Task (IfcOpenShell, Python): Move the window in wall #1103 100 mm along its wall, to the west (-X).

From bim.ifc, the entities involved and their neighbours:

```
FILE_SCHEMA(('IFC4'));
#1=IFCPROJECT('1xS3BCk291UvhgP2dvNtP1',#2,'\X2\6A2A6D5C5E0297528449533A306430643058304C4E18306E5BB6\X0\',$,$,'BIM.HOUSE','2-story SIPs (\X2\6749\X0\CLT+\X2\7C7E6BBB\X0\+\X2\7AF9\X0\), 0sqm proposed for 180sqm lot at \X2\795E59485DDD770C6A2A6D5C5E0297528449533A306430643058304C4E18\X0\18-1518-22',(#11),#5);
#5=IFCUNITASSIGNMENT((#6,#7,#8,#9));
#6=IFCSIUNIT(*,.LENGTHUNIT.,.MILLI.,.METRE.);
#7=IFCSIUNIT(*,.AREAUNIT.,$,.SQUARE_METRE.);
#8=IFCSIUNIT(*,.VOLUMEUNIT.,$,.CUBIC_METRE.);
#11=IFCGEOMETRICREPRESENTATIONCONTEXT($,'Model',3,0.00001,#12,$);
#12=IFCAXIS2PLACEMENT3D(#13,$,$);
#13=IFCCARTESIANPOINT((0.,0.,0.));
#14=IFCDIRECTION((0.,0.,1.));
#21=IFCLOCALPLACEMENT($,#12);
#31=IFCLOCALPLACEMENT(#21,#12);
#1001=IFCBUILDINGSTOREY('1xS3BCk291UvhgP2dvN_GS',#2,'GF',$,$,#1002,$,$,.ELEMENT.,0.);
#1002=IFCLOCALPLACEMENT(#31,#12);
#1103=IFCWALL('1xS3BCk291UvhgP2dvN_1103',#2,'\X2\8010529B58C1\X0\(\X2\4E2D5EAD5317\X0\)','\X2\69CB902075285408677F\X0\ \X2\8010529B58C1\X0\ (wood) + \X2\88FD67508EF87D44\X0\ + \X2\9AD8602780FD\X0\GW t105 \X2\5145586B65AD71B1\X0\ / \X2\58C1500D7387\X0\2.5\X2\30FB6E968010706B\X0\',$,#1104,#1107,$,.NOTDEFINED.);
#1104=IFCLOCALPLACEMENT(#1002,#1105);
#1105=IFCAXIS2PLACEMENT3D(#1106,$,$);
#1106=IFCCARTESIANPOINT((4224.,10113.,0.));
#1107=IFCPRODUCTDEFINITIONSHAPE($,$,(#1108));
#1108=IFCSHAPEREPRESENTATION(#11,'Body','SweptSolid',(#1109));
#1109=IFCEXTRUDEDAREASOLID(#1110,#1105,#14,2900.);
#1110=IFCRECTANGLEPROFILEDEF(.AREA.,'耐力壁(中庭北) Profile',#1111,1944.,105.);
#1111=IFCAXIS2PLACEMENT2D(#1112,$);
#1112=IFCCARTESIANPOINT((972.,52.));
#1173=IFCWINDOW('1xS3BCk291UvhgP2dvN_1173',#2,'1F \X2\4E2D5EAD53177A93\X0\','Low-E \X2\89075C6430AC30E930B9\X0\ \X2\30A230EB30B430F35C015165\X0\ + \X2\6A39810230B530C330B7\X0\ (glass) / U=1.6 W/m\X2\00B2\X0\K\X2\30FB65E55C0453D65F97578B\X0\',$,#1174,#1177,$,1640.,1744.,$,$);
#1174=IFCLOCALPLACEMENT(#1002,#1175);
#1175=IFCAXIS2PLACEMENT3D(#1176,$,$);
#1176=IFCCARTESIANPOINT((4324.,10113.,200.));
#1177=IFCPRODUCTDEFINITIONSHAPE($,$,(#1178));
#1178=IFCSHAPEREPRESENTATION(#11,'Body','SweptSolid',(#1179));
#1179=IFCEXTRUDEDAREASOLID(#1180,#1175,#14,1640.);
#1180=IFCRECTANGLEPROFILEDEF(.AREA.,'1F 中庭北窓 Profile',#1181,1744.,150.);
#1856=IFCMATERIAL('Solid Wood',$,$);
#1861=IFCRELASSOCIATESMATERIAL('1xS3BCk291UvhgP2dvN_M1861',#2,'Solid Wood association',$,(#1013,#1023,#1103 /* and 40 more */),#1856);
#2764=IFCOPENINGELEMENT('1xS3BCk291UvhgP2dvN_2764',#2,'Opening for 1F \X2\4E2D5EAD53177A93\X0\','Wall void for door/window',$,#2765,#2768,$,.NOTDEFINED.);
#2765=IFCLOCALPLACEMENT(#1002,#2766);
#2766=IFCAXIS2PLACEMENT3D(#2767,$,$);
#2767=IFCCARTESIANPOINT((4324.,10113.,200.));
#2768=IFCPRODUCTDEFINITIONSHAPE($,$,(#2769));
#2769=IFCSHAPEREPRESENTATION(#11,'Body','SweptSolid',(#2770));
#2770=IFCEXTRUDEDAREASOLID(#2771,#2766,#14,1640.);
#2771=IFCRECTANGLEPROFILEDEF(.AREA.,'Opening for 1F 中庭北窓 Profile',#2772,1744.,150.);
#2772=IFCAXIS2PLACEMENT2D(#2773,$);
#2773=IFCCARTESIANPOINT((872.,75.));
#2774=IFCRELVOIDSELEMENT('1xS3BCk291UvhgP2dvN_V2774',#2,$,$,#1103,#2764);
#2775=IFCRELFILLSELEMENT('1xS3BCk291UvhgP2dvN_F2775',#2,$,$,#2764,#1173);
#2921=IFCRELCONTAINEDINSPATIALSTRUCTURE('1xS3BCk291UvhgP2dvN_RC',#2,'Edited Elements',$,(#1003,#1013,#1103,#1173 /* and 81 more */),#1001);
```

```python
import ifcopenshell
import ifcopenshell.api.geometry
import ifcopenshell.util.placement
import ifcopenshell.util.unit

model = ifcopenshell.open("bim.ifc")
unit_scale = ifcopenshell.util.unit.calculate_unit_scale(model)

window = model.by_id(1173)
opening = window.FillsVoids[0].RelatingOpeningElement
wall = opening.VoidsElements[0].RelatingBuildingElement

wall_matrix = ifcopenshell.util.placement.get_local_placement(wall.ObjectPlacement)
shift = wall_matrix[:3, 0] * -0.1 / unit_scale
before = ifcopenshell.util.placement.get_local_placement(window.ObjectPlacement)[:3, 3].copy()

# The window is not placed relative to its opening, so move both.
for product in (opening, window):
    matrix = ifcopenshell.util.placement.get_local_placement(product.ObjectPlacement)
    matrix[:3, 3] += shift
    ifcopenshell.api.geometry.edit_object_placement(model, product=product, matrix=matrix, is_si=False)

after = ifcopenshell.util.placement.get_local_placement(window.ObjectPlacement)[:3, 3]
print("window moved by", (after - before).round(3) + 0.0)

model.write("bim_rev.ifc")
```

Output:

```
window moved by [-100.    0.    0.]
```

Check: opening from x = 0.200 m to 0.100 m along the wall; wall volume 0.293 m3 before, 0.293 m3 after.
